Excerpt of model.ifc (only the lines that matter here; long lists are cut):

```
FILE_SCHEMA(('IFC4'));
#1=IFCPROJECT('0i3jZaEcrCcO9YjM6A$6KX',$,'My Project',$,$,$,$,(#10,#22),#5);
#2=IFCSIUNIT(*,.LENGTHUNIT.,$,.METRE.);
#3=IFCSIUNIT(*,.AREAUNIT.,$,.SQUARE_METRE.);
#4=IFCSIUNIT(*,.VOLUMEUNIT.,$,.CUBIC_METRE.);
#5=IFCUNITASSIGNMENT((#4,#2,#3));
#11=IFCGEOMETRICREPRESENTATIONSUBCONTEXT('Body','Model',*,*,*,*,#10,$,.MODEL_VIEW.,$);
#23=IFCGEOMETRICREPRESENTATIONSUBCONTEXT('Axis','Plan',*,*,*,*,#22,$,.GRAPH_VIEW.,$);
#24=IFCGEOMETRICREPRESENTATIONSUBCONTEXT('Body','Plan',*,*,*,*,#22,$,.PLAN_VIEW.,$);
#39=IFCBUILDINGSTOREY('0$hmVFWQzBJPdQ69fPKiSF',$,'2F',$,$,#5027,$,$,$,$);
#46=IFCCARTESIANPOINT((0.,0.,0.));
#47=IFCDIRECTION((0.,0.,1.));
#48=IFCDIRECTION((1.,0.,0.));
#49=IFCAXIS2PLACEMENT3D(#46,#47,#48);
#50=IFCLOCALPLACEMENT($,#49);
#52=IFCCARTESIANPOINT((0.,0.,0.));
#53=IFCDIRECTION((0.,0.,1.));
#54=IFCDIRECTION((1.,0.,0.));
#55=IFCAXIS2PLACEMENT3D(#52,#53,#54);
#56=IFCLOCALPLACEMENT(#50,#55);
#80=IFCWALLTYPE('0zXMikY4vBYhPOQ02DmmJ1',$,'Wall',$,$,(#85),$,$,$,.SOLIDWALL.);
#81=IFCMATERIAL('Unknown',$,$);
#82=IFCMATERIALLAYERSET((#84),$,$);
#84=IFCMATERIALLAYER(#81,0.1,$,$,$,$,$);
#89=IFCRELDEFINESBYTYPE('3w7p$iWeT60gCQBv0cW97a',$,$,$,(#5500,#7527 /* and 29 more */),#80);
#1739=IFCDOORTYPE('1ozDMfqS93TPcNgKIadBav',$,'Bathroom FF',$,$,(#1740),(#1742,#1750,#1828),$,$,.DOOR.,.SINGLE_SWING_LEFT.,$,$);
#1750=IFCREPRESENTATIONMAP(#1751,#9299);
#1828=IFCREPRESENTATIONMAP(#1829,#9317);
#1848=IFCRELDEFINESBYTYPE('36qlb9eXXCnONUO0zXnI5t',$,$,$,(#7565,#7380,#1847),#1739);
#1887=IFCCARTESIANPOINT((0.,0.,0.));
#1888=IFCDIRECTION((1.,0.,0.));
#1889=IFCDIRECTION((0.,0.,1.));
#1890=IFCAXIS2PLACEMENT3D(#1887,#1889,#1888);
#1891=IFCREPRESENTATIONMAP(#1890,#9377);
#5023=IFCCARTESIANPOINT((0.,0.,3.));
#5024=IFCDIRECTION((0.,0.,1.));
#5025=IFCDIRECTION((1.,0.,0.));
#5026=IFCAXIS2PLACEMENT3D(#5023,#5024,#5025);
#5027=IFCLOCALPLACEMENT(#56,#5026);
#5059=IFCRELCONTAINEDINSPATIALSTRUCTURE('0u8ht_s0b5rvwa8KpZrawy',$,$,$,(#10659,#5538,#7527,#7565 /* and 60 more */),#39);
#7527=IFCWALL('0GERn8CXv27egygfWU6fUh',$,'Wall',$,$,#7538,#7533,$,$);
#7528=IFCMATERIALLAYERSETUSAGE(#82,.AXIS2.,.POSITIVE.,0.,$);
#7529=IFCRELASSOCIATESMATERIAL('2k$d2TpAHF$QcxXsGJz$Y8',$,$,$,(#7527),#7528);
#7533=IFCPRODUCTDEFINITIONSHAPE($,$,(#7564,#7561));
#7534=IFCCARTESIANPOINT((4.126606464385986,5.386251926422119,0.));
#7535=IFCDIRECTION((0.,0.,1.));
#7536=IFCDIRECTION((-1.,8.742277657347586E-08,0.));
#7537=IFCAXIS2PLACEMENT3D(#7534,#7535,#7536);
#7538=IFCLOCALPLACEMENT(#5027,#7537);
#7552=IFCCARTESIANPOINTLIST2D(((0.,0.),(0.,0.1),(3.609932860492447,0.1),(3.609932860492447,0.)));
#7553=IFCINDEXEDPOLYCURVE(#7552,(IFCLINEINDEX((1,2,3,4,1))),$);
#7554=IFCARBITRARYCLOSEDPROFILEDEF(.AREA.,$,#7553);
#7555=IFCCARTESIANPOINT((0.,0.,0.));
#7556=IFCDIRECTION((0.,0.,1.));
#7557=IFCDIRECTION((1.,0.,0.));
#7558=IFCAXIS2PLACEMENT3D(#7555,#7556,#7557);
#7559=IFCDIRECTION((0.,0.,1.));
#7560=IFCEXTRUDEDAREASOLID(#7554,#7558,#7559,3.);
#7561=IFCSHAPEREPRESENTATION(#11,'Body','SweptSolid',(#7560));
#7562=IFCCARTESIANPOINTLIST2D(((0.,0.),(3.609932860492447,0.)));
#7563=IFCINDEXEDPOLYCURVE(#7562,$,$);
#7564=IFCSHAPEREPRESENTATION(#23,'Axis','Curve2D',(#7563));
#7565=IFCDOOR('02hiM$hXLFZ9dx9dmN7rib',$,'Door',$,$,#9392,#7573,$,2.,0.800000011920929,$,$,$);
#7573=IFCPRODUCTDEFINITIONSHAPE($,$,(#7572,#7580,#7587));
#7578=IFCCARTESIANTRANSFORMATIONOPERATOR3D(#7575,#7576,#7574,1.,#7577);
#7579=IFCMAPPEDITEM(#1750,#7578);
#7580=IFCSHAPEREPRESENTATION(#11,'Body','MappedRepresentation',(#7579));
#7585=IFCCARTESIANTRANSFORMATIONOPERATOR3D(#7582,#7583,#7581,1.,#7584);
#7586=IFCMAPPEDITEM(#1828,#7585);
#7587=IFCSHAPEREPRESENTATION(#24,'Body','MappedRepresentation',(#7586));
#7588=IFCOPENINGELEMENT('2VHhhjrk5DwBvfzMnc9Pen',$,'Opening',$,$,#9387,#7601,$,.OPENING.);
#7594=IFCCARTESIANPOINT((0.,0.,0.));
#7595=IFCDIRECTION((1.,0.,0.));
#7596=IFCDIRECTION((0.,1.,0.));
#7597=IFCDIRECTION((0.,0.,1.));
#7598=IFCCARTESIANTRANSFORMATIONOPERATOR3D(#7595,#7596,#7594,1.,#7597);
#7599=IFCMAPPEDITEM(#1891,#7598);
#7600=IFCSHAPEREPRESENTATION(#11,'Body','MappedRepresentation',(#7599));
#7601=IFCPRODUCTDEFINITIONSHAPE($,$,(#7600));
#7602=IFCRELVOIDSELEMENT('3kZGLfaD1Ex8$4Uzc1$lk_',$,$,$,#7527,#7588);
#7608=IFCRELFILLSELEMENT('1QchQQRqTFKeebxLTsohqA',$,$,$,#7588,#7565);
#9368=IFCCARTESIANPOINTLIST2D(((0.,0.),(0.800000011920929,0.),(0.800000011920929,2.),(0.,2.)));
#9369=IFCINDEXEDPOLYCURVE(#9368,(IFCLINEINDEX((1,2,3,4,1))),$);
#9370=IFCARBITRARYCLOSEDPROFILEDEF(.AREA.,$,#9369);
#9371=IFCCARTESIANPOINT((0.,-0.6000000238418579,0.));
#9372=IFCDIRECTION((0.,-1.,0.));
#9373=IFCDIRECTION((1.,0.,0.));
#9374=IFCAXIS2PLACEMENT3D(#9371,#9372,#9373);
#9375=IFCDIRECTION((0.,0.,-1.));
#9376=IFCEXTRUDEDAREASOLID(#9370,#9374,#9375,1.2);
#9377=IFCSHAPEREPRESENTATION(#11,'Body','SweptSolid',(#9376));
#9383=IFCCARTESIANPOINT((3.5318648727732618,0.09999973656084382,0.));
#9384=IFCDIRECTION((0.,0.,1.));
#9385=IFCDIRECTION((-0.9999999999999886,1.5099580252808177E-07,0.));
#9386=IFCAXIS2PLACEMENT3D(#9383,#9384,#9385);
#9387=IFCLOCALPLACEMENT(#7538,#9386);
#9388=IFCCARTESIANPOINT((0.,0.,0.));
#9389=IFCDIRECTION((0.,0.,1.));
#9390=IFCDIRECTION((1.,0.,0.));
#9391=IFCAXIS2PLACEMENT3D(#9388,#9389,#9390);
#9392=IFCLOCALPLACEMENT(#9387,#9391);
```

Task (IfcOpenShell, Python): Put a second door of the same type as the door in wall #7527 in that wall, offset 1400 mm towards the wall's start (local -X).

```python
import ifcopenshell
import ifcopenshell.api.feature
import ifcopenshell.api.geometry
import ifcopenshell.api.root
import ifcopenshell.geom
import ifcopenshell.util.element
import ifcopenshell.util.placement
import ifcopenshell.util.shape
import ifcopenshell.util.unit

model = ifcopenshell.open("model.ifc")
unit_scale = ifcopenshell.util.unit.calculate_unit_scale(model)
settings = ifcopenshell.geom.settings()


def volume(element):
    """Net volume in cubic metres, openings subtracted."""
    shape = ifcopenshell.geom.create_shape(settings, element)
    return ifcopenshell.util.shape.get_volume(shape.geometry)


door = model.by_guid("02hiM$hXLFZ9dx9dmN7rib")
opening = door.FillsVoids[0].RelatingOpeningElement
wall = opening.VoidsElements[0].RelatingBuildingElement
before = volume(wall)
shift = ifcopenshell.util.placement.get_local_placement(wall.ObjectPlacement)[:3, 0] * -1.4 / unit_scale

# copy_class copies the void relationship, type, container and properties, but no geometry.
new_opening = ifcopenshell.api.root.copy_class(model, product=opening)
new_opening.Representation = ifcopenshell.util.element.copy_deep(
    model, opening.Representation, exclude=["IfcGeometricRepresentationContext", "IfcRepresentationMap"]
)
new_door = ifcopenshell.api.root.copy_class(model, product=door)
new_door.Representation = ifcopenshell.util.element.copy_deep(
    model, door.Representation, exclude=["IfcGeometricRepresentationContext", "IfcRepresentationMap"]
)
ifcopenshell.api.feature.add_filling(model, opening=new_opening, element=new_door)

for old, new in ((opening, new_opening), (door, new_door)):
    matrix = ifcopenshell.util.placement.get_local_placement(old.ObjectPlacement)
    matrix[:3, 3] += shift
    ifcopenshell.api.geometry.edit_object_placement(model, product=new, matrix=matrix, is_si=False)

after = volume(wall)

print(f"wall volume {before:.3f} -> {after:.3f} m3")

model.write("model-out.ifc")
```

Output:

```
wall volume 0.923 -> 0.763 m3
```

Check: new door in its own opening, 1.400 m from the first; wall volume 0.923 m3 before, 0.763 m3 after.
